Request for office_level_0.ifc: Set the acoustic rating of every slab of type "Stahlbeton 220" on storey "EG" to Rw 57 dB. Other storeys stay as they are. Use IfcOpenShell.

First a look at what the model holds.

```python
import ifcopenshell
import ifcopenshell.util.element

model = ifcopenshell.open("office_level_0.ifc")
print(model.schema)
storey = next(s for s in model.by_type("IfcBuildingStorey") if s.Name == "EG")
slabs = [e for e in ifcopenshell.util.element.get_decomposition(storey) if e.is_a("IfcSlab")]
seen = {}
for e in slabs:
    element_type = ifcopenshell.util.element.get_type(e)
    key = (element_type.Name if element_type != e and element_type else None, ifcopenshell.util.element.get_pset(e, "Pset_SlabCommon", "AcousticRating"))
    seen[key] = seen.get(key, 0) + 1
for (name, value), count in sorted(seen.items(), key=str):
    print(count, "x", name, "|", value)
```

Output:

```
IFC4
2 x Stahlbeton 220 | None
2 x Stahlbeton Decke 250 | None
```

```python
import ifcopenshell
import ifcopenshell.api.pset
import ifcopenshell.util.element

model = ifcopenshell.open("office_level_0.ifc")

storey = next(s for s in model.by_type("IfcBuildingStorey") if s.Name == "EG")
slabs = [e for e in ifcopenshell.util.element.get_decomposition(storey) if e.is_a("IfcSlab")]

count = 0
for e in slabs:
    element_type = ifcopenshell.util.element.get_type(e)
    if element_type in (None, e) or element_type.Name != "Stahlbeton 220":
        continue
    # add_pset returns the element's existing set when there is one.
    pset = ifcopenshell.api.pset.add_pset(model, product=e, name="Pset_SlabCommon")
    ifcopenshell.api.pset.edit_pset(model, pset=pset, properties={"AcousticRating": "Rw 57 dB"})
    count += 1

print(count, "slabs updated")

model.write("office_level_0-out.ifc")
```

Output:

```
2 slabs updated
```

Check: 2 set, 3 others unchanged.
